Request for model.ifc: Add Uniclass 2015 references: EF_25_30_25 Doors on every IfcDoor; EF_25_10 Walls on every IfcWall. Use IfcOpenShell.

First a look at what the model holds.

```python
import ifcopenshell

model = ifcopenshell.open("model.ifc")
print(model.schema)
print("classifications:", [c.Name for c in model.by_type("IfcClassification")])
for ifc_class in ("IfcDoor", "IfcRoof", "IfcStair", "IfcWall", "IfcWindow"):
    print(ifc_class, len(model.by_type(ifc_class)))
```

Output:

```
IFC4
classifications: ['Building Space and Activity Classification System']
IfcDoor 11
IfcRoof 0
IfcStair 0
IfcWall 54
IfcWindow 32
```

```python
import ifcopenshell
import ifcopenshell.api.classification

model = ifcopenshell.open("model.ifc")

system = ifcopenshell.api.classification.add_classification(model, classification="Uniclass 2015")

codes = {
    "IfcDoor": ("EF_25_30_25", "Doors"),
    "IfcWall": ("EF_25_10", "Walls"),
}
for ifc_class, (code, name) in codes.items():
    products = model.by_type(ifc_class)
    ifcopenshell.api.classification.add_reference(
        model, products=products, classification=system, identification=code, name=name
    )
    print(code, len(products))

model.write("model-out.ifc")
```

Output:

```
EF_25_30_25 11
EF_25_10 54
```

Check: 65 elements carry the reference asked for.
